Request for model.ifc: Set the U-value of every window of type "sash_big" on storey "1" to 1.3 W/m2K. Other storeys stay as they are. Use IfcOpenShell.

First a look at what the model holds.

```python
import ifcopenshell
import ifcopenshell.util.element

model = ifcopenshell.open("model.ifc")
print(model.schema)
storey = next(s for s in model.by_type("IfcBuildingStorey") if s.Name == "1")
windows = [e for e in ifcopenshell.util.element.get_decomposition(storey) if e.is_a("IfcWindow")]
seen = {}
for e in windows:
    element_type = ifcopenshell.util.element.get_type(e)
    key = (element_type.Name if element_type != e and element_type else None, ifcopenshell.util.element.get_pset(e, "Pset_WindowCommon", "ThermalTransmittance"))
    seen[key] = seen.get(key, 0) + 1
for (name, value), count in sorted(seen.items(), key=str):
    print(count, "x", name, "|", value)
```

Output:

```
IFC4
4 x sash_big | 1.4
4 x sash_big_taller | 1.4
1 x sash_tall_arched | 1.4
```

```python
import ifcopenshell
import ifcopenshell.api.pset
import ifcopenshell.util.element

model = ifcopenshell.open("model.ifc")

storey = next(s for s in model.by_type("IfcBuildingStorey") if s.Name == "1")
windows = [e for e in ifcopenshell.util.element.get_decomposition(storey) if e.is_a("IfcWindow")]

count = 0
for e in windows:
    element_type = ifcopenshell.util.element.get_type(e)
    if element_type in (None, e) or element_type.Name != "sash_big":
        continue
    # add_pset returns the element's existing set when there is one.
    pset = ifcopenshell.api.pset.add_pset(model, product=e, name="Pset_WindowCommon")
    ifcopenshell.api.pset.edit_pset(model, pset=pset, properties={"ThermalTransmittance": 1.3})
    count += 1

print(count, "windows updated")

model.write("model_rev.ifc")
```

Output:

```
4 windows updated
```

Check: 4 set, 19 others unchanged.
